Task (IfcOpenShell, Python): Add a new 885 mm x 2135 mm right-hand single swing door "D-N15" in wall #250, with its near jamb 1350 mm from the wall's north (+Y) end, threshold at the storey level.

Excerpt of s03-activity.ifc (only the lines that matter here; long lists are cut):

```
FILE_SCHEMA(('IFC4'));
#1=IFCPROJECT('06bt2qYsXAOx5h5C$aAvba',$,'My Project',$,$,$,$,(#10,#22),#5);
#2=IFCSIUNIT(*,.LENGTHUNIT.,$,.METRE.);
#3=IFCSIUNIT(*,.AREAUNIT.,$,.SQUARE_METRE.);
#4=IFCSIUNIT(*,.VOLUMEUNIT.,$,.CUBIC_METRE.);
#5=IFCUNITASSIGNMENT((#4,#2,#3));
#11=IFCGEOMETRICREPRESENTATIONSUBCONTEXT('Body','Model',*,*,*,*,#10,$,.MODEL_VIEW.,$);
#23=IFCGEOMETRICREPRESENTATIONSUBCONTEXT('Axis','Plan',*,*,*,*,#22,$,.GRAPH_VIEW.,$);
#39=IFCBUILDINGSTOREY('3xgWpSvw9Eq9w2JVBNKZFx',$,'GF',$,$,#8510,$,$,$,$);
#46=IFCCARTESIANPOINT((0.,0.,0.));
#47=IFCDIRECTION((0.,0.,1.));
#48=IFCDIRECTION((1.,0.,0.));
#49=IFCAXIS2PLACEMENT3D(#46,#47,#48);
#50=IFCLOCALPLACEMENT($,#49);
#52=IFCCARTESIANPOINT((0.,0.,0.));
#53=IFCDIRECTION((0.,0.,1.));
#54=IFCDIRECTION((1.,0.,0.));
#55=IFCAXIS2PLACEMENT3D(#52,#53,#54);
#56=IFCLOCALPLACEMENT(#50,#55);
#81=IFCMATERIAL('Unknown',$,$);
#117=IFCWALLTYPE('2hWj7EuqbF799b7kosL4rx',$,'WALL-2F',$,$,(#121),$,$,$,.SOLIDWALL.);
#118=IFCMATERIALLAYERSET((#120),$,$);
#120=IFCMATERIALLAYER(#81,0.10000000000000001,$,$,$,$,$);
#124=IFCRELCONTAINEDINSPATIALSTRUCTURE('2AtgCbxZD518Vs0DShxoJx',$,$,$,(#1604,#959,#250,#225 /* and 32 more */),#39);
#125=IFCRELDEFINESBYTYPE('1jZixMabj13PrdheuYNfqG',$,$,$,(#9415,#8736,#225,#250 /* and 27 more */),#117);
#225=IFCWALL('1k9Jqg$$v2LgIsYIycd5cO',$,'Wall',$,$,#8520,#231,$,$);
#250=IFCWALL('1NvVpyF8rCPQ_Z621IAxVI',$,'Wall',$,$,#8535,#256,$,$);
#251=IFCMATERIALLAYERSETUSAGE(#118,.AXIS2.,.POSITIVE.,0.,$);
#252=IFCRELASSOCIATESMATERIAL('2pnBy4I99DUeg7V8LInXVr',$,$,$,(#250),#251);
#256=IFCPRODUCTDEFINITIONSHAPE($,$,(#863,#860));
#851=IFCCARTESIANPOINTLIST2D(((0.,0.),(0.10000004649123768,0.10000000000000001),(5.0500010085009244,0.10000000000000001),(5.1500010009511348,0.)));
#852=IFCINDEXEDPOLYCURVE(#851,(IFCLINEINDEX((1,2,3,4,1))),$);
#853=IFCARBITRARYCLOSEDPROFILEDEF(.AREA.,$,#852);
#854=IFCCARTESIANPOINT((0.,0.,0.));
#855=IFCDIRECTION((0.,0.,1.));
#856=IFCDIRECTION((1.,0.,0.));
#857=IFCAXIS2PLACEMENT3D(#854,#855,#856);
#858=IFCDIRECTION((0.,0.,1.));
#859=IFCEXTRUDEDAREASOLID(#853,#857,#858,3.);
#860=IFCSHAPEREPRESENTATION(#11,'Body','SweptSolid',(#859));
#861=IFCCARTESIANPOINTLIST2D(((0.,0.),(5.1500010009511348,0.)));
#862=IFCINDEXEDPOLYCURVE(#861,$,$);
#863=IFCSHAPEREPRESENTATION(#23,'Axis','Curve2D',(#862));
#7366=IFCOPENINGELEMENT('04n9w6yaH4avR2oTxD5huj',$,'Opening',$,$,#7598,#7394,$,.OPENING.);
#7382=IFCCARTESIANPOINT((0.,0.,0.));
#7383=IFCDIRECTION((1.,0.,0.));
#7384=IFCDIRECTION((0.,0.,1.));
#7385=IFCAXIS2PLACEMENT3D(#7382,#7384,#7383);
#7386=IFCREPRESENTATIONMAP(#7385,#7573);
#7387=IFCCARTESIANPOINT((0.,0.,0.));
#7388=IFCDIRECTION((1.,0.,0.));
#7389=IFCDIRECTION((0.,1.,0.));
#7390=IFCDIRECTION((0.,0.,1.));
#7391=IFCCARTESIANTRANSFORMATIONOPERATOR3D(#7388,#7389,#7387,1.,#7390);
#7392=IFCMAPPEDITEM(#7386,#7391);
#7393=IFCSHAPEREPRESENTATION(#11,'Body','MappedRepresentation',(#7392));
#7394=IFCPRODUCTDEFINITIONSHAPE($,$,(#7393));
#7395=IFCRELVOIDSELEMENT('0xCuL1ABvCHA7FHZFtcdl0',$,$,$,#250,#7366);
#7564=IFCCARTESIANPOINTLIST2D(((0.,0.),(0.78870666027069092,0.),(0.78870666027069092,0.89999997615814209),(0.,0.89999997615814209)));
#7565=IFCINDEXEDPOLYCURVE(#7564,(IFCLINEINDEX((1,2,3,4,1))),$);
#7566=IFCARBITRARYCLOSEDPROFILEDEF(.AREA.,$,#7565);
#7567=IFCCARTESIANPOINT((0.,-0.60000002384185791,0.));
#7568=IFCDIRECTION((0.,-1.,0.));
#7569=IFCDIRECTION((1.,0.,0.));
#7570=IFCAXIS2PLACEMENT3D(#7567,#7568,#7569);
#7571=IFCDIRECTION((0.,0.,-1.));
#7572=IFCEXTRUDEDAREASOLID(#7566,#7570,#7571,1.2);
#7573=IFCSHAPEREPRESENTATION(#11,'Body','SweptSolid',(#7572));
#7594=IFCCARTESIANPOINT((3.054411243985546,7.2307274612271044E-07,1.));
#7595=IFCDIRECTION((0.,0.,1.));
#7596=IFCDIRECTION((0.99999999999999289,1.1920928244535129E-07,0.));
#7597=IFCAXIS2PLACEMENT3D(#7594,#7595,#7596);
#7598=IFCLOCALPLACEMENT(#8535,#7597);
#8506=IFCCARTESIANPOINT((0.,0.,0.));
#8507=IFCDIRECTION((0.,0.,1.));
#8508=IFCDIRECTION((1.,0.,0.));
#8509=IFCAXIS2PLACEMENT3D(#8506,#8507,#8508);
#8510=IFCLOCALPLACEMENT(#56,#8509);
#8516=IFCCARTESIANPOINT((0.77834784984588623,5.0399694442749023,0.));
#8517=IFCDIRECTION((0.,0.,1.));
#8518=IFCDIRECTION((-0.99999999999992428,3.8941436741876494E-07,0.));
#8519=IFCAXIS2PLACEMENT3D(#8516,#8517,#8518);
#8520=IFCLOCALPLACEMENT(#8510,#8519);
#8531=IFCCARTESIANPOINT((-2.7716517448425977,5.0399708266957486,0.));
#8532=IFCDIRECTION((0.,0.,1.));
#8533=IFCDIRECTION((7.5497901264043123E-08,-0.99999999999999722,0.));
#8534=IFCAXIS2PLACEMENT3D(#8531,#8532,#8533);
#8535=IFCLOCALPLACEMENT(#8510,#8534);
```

```python
import numpy as np
import ifcopenshell
import ifcopenshell.api.feature
import ifcopenshell.api.geometry
import ifcopenshell.api.root
import ifcopenshell.api.spatial
import ifcopenshell.geom
import ifcopenshell.util.element
import ifcopenshell.util.placement
import ifcopenshell.util.representation
import ifcopenshell.util.shape
import ifcopenshell.util.unit

model = ifcopenshell.open("s03-activity.ifc")
unit_scale = ifcopenshell.util.unit.calculate_unit_scale(model)
settings = ifcopenshell.geom.settings()


def volume(element):
    """Net volume in cubic metres, openings subtracted."""
    shape = ifcopenshell.geom.create_shape(settings, element)
    return ifcopenshell.util.shape.get_volume(shape.geometry)


wall = model.by_id(250)
storey = ifcopenshell.util.element.get_container(wall, ifc_class="IfcBuildingStorey")
context = ifcopenshell.util.representation.get_context(model, "Model", "Body", "MODEL_VIEW")
before = volume(wall)

width, height, from_end, sill = 0.885, 2.135, 1.35, 0.0  # metres

# The wall runs along its own X axis, and the end named is its -X end.
wall_shape = ifcopenshell.geom.create_shape(settings, wall)
x, y, z = ifcopenshell.util.shape.get_vertices(wall_shape.geometry).T
start = x.min() + from_end
face, thickness = float(y.min()), float(y.max() - y.min())
wall_matrix = ifcopenshell.util.placement.get_local_placement(wall.ObjectPlacement)
level = ifcopenshell.util.placement.get_local_placement(storey.ObjectPlacement)[2, 3]


def in_wall(x, y):
    """Placement at x, y metres in the wall's axes, at sill height."""
    matrix = wall_matrix.copy()
    matrix[:, 3] = wall_matrix @ np.array([x / unit_scale, y / unit_scale, 0.0, 1.0])
    matrix[2, 3] = level + sill / unit_scale
    return matrix


# Opening: a box that overshoots both wall faces by 50 mm.
opening = ifcopenshell.api.root.create_entity(model, ifc_class="IfcOpeningElement", predefined_type="OPENING")
box = ifcopenshell.api.geometry.add_wall_representation(
    model, context=context, length=width, height=height, thickness=thickness + 0.1
)
ifcopenshell.api.geometry.assign_representation(model, product=opening, representation=box)
ifcopenshell.api.geometry.edit_object_placement(model, product=opening, matrix=in_wall(start, face - 0.05), is_si=False)
ifcopenshell.api.feature.add_feature(model, feature=opening, element=wall)

door = ifcopenshell.api.root.create_entity(model, ifc_class="IfcDoor", name="D-N15", predefined_type="DOOR")
door.OverallWidth, door.OverallHeight = width / unit_scale, height / unit_scale
door.OperationType = "SINGLE_SWING_RIGHT"
body = ifcopenshell.api.geometry.add_door_representation(
    model,
    context=context,
    overall_width=door.OverallWidth,
    overall_height=door.OverallHeight,
    operation_type="SINGLE_SWING_RIGHT",
    lining_properties={"LiningDepth": thickness / unit_scale, "ThresholdDepth": thickness / unit_scale},
)
ifcopenshell.api.geometry.assign_representation(model, product=door, representation=body)
ifcopenshell.api.spatial.assign_container(model, products=[door], relating_structure=storey)
ifcopenshell.api.feature.add_filling(model, opening=opening, element=door)

# The lining spans the wall, so the door starts at the wall face.
ifcopenshell.api.geometry.edit_object_placement(model, product=door, matrix=in_wall(start, face), is_si=False)

after = volume(wall)

print(f"wall volume {before:.3f} -> {after:.3f} m3")

model.write("s03-activity_rev.ifc")
```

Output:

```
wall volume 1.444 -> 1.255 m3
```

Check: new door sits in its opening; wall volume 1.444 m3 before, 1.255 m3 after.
